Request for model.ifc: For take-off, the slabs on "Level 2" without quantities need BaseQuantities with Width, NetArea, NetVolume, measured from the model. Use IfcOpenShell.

First a look at what the model holds.

```python
import ifcopenshell
import ifcopenshell.util.element
import ifcopenshell.util.unit

model = ifcopenshell.open("model.ifc")
print(model.schema)
for unit_type in ("LENGTHUNIT", "AREAUNIT", "VOLUMEUNIT"):
    print(unit_type, ifcopenshell.util.unit.calculate_unit_scale(model, unit_type))
storey = next(s for s in model.by_type("IfcBuildingStorey") if s.Name == "Level 2")
slabs = [e for e in ifcopenshell.util.element.get_decomposition(storey) if e.is_a("IfcSlab")]
for e in sorted(slabs, key=lambda e: e.id()):
    print(e.id(), e.is_a(), e.Name, list(ifcopenshell.util.element.get_psets(e, qtos_only=True)), sep=" | ")
```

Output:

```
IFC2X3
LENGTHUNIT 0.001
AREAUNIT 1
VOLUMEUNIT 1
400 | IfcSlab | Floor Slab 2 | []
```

```python
import ifcopenshell
import ifcopenshell.api.pset
import ifcopenshell.geom
import ifcopenshell.util.element
import ifcopenshell.util.shape
import ifcopenshell.util.unit

model = ifcopenshell.open("model.ifc")
unit_scale = ifcopenshell.util.unit.calculate_unit_scale(model)
area_scale = ifcopenshell.util.unit.calculate_unit_scale(model, "AREAUNIT")
volume_scale = ifcopenshell.util.unit.calculate_unit_scale(model, "VOLUMEUNIT")
settings = ifcopenshell.geom.settings()

storey = next(s for s in model.by_type("IfcBuildingStorey") if s.Name == "Level 2")
slabs = [e for e in ifcopenshell.util.element.get_decomposition(storey) if e.is_a("IfcSlab")]

for e in sorted(slabs, key=lambda e: e.id()):
    if ifcopenshell.util.element.get_psets(e, qtos_only=True, should_inherit=False):
        continue
    # Geometry comes back in metres, in the element's own axes.
    shape = ifcopenshell.geom.create_shape(settings, e)
    values = {
        "Width": ifcopenshell.util.shape.get_z(shape.geometry) / unit_scale,
        "NetArea": ifcopenshell.util.shape.get_footprint_area(shape.geometry) / area_scale,
        "NetVolume": ifcopenshell.util.shape.get_volume(shape.geometry) / volume_scale,
    }
    qto = ifcopenshell.api.pset.add_qto(model, product=e, name="BaseQuantities")
    ifcopenshell.api.pset.edit_qto(model, qto=qto, properties=values)
    print(e.id(), {k: round(v, 3) for k, v in values.items()})

model.write("model_edited.ifc")
```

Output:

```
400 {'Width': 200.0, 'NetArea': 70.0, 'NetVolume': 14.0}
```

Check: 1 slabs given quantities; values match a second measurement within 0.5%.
